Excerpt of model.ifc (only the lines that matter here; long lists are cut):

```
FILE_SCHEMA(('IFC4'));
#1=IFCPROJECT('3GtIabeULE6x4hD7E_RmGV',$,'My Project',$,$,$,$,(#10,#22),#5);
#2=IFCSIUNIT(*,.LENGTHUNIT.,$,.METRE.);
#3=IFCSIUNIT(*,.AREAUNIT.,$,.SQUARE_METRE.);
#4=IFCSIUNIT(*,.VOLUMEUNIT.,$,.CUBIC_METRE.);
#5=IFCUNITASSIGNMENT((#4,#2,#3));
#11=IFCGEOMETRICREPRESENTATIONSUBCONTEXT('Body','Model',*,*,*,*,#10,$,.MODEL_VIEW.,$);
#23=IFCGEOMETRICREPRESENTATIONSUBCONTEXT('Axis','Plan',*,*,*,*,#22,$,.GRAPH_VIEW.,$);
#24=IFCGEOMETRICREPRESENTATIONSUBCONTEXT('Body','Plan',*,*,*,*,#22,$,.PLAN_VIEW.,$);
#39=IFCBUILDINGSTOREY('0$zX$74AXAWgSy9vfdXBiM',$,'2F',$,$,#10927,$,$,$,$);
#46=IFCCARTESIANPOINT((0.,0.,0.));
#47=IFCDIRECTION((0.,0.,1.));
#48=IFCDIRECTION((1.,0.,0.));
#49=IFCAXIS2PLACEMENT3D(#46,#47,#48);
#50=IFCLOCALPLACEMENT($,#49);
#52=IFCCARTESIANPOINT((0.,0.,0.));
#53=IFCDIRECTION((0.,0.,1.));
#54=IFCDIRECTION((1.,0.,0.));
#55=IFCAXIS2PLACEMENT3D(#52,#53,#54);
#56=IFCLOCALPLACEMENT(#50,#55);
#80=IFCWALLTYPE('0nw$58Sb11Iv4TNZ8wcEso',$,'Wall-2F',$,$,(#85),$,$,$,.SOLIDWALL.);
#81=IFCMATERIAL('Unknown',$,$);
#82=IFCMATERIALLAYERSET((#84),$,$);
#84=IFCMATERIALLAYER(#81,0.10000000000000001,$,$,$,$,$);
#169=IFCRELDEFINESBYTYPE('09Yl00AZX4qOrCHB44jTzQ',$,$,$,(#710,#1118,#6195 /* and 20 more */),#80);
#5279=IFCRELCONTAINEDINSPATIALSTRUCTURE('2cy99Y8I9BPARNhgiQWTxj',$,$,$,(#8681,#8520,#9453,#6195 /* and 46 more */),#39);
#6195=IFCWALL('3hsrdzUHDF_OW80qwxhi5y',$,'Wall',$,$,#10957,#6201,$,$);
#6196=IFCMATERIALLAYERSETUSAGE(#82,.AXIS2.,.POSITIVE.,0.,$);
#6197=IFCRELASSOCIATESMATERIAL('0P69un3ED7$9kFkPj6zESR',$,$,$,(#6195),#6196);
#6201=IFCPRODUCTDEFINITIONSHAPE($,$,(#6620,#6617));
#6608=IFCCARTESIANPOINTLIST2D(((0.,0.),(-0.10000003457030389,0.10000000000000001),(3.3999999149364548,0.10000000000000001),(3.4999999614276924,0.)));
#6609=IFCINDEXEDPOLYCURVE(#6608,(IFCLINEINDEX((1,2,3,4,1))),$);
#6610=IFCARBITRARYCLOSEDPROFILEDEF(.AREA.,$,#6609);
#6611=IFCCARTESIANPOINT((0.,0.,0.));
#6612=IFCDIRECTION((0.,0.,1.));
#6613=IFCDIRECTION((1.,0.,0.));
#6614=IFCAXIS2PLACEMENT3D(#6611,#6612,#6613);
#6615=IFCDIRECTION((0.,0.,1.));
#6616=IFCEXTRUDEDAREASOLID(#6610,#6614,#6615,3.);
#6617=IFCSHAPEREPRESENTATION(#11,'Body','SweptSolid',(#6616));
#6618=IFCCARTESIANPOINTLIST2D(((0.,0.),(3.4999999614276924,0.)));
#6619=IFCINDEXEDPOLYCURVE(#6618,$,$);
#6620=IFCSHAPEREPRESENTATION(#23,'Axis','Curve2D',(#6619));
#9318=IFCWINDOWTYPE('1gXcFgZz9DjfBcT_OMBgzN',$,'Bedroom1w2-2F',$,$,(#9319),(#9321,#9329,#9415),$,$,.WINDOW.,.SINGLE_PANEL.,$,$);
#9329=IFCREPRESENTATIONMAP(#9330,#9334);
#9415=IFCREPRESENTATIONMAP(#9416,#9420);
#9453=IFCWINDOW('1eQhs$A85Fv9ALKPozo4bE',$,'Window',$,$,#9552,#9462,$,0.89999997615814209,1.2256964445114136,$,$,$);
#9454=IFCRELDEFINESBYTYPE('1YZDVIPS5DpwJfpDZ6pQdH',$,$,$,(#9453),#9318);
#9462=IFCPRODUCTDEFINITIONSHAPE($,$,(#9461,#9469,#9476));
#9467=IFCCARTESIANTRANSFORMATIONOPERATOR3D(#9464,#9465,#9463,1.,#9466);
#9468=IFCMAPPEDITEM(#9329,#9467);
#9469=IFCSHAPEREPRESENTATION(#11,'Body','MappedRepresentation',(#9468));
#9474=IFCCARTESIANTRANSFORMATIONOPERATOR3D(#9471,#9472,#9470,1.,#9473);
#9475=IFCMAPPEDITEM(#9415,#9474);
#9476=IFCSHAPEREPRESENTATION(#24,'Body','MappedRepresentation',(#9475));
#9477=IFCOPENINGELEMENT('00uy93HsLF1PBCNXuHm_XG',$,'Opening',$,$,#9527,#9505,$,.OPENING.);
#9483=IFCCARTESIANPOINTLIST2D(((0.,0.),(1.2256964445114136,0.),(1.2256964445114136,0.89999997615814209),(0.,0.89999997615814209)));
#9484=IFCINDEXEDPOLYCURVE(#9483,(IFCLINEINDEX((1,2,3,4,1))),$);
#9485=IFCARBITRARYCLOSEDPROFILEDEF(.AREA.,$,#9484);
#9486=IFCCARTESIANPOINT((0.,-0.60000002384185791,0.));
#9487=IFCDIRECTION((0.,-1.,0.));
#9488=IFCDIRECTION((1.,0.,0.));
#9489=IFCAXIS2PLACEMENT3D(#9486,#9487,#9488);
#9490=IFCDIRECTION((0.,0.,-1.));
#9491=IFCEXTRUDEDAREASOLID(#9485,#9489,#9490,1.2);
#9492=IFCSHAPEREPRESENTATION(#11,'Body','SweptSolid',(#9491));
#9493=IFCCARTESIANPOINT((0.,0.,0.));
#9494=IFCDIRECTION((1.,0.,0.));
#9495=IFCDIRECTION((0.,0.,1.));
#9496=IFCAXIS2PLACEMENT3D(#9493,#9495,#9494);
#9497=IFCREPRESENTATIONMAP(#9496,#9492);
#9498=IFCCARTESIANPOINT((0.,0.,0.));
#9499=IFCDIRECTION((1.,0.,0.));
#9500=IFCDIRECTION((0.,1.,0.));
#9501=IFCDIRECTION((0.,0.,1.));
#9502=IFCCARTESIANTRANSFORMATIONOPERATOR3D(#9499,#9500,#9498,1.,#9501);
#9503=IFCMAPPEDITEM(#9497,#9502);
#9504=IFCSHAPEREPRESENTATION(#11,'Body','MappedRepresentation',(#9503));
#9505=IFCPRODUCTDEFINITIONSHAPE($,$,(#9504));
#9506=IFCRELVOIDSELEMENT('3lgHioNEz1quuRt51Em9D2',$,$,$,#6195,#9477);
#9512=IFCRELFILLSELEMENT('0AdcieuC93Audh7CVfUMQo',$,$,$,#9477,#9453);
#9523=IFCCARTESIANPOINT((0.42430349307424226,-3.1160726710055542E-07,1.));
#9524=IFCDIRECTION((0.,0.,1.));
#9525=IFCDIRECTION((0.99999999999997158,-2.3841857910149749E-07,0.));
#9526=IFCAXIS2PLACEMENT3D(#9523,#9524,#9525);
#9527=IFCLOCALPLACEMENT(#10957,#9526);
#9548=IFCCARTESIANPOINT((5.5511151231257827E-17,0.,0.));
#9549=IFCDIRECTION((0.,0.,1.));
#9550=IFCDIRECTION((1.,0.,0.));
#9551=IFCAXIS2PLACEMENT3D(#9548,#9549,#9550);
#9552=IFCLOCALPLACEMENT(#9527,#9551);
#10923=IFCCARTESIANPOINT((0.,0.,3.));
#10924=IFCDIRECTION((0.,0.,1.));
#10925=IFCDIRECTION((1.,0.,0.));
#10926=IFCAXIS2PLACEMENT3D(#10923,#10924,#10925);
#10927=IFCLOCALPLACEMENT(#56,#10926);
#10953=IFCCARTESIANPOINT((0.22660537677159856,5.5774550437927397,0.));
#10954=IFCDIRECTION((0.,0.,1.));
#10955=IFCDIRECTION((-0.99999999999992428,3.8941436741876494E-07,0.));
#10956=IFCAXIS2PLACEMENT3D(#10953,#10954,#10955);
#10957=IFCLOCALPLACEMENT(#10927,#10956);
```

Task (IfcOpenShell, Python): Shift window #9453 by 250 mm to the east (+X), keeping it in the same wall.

```python
import ifcopenshell
import ifcopenshell.api.geometry
import ifcopenshell.util.placement

model = ifcopenshell.open("model.ifc")

window = model.by_id(9453)
opening = window.FillsVoids[0].RelatingOpeningElement
wall = opening.VoidsElements[0].RelatingBuildingElement

wall_matrix = ifcopenshell.util.placement.get_local_placement(wall.ObjectPlacement)
shift = wall_matrix[:3, 0] * -0.25
before = ifcopenshell.util.placement.get_local_placement(window.ObjectPlacement)[:3, 3].copy()

# The window is placed relative to its opening, so it follows when the opening moves.
matrix = ifcopenshell.util.placement.get_local_placement(opening.ObjectPlacement)
matrix[:3, 3] += shift
ifcopenshell.api.geometry.edit_object_placement(
    model, product=opening, matrix=matrix, is_si=False, should_transform_children=True
)

after = ifcopenshell.util.placement.get_local_placement(window.ObjectPlacement)[:3, 3]
print("window moved by", (after - before).round(3) + 0.0)

model.write("model_updated.ifc")
```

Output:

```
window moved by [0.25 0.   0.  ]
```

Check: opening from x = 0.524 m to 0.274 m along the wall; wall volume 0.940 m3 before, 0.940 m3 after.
